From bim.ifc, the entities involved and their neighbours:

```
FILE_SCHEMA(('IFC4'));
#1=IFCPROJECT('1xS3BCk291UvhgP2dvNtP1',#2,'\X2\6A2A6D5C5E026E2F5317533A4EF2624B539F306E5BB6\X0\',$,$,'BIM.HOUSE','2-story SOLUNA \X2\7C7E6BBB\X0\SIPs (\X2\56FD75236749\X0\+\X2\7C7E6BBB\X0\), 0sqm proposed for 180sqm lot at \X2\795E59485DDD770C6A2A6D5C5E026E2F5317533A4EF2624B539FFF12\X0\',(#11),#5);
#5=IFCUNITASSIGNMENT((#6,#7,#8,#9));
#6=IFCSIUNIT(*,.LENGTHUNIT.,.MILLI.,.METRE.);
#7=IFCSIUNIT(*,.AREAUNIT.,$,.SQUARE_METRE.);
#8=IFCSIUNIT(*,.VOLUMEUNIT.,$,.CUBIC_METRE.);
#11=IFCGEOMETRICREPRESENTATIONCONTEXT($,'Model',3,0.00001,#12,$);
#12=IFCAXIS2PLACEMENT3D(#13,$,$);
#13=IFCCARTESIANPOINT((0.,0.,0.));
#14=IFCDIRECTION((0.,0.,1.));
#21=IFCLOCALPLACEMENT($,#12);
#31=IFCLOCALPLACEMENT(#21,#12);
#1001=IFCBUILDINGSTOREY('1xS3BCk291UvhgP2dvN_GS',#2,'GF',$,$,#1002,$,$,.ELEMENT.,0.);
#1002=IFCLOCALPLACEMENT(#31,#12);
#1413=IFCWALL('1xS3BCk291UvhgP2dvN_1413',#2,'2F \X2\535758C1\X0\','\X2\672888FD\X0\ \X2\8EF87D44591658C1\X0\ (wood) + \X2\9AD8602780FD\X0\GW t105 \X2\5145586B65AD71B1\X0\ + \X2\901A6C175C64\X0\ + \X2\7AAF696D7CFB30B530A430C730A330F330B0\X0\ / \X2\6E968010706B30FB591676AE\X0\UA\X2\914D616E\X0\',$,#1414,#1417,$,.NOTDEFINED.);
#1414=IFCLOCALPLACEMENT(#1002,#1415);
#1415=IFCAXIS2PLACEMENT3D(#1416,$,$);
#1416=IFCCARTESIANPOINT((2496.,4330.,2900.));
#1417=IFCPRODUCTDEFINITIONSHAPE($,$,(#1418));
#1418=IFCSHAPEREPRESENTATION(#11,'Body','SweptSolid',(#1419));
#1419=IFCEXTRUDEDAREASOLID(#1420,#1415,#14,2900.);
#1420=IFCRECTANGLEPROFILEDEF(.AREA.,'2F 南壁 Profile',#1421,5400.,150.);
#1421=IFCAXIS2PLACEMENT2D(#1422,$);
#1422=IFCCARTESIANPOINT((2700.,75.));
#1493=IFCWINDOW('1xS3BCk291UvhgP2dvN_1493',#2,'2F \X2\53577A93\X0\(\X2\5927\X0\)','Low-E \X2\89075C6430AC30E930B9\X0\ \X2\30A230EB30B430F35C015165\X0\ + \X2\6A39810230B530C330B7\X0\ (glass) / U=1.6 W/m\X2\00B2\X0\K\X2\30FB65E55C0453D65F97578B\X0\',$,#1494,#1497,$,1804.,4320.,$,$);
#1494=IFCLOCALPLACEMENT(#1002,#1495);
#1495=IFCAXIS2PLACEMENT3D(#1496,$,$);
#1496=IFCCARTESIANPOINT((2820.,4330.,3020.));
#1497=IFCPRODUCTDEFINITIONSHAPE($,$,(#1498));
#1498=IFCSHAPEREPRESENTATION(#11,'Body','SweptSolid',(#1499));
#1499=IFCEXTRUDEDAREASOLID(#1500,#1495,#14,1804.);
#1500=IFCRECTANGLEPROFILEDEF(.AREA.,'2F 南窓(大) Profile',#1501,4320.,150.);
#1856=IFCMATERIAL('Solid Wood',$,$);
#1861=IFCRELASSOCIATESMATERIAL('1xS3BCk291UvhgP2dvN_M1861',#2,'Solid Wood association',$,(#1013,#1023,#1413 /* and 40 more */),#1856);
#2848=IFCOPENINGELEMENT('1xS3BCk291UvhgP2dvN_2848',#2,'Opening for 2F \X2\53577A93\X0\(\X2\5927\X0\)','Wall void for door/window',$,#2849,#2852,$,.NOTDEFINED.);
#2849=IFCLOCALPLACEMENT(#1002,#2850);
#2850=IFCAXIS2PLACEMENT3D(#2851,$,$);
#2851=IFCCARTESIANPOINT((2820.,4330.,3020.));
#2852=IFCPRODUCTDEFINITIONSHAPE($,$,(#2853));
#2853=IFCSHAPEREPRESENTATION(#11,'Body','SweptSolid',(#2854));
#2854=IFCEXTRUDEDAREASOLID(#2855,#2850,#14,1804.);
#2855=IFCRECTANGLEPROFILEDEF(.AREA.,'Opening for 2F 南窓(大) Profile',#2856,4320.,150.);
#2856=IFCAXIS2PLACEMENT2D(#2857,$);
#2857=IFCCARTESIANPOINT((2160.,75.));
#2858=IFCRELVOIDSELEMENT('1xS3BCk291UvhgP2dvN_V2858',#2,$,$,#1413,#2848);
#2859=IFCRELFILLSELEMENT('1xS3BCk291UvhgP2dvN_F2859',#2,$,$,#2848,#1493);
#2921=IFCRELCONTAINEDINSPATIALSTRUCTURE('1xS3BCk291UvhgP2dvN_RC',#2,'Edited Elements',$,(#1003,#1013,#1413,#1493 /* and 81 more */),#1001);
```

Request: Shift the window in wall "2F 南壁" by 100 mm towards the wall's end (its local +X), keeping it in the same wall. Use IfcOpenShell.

```python
import ifcopenshell
import ifcopenshell.api.geometry
import ifcopenshell.util.placement
import ifcopenshell.util.unit

model = ifcopenshell.open("bim.ifc")
unit_scale = ifcopenshell.util.unit.calculate_unit_scale(model)

window = model.by_id(1493)
opening = window.FillsVoids[0].RelatingOpeningElement
wall = opening.VoidsElements[0].RelatingBuildingElement

wall_matrix = ifcopenshell.util.placement.get_local_placement(wall.ObjectPlacement)
shift = wall_matrix[:3, 0] * 0.1 / unit_scale
before = ifcopenshell.util.placement.get_local_placement(window.ObjectPlacement)[:3, 3].copy()

# The window is not placed relative to its opening, so move both.
for product in (opening, window):
    matrix = ifcopenshell.util.placement.get_local_placement(product.ObjectPlacement)
    matrix[:3, 3] += shift
    ifcopenshell.api.geometry.edit_object_placement(model, product=product, matrix=matrix, is_si=False)

after = ifcopenshell.util.placement.get_local_placement(window.ObjectPlacement)[:3, 3]
print("window moved by", (after - before).round(3) + 0.0)

model.write("bim_edited.ifc")
```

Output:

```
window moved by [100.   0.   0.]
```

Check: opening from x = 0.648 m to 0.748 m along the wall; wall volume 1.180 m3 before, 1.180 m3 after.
